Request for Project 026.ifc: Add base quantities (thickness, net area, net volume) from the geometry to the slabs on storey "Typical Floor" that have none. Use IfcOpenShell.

First a look at what the model holds.

```python
import ifcopenshell
import ifcopenshell.util.element
import ifcopenshell.util.unit

model = ifcopenshell.open("Project 026.ifc")
print(model.schema)
for unit_type in ("LENGTHUNIT", "AREAUNIT", "VOLUMEUNIT"):
    print(unit_type, ifcopenshell.util.unit.calculate_unit_scale(model, unit_type))
storey = next(s for s in model.by_type("IfcBuildingStorey") if s.Name == "Typical Floor")
slabs = [e for e in ifcopenshell.util.element.get_decomposition(storey) if e.is_a("IfcSlab")]
for e in sorted(slabs, key=lambda e: e.id()):
    print(e.id(), e.is_a(), e.Name, list(ifcopenshell.util.element.get_psets(e, qtos_only=True)), sep=" | ")
```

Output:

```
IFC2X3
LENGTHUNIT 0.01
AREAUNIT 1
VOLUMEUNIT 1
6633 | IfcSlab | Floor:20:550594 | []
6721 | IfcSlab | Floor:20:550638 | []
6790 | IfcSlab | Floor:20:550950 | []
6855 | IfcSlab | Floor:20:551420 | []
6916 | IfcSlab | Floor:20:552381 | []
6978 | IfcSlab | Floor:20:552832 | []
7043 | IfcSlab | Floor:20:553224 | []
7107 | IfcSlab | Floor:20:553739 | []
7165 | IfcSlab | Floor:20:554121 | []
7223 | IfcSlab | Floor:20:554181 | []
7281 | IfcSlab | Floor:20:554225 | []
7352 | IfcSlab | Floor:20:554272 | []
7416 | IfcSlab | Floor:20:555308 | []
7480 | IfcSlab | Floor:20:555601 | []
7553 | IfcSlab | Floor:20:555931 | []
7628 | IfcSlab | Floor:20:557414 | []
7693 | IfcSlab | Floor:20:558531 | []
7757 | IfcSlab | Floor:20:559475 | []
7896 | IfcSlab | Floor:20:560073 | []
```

```python
import ifcopenshell
import ifcopenshell.api.pset
import ifcopenshell.geom
import ifcopenshell.util.element
import ifcopenshell.util.shape
import ifcopenshell.util.unit

model = ifcopenshell.open("Project 026.ifc")
unit_scale = ifcopenshell.util.unit.calculate_unit_scale(model)
area_scale = ifcopenshell.util.unit.calculate_unit_scale(model, "AREAUNIT")
volume_scale = ifcopenshell.util.unit.calculate_unit_scale(model, "VOLUMEUNIT")
settings = ifcopenshell.geom.settings()

storey = next(s for s in model.by_type("IfcBuildingStorey") if s.Name == "Typical Floor")
slabs = [e for e in ifcopenshell.util.element.get_decomposition(storey) if e.is_a("IfcSlab")]

for e in sorted(slabs, key=lambda e: e.id()):
    if ifcopenshell.util.element.get_psets(e, qtos_only=True, should_inherit=False):
        continue
    # Geometry comes back in metres, in the element's own axes.
    shape = ifcopenshell.geom.create_shape(settings, e)
    values = {
        "Width": ifcopenshell.util.shape.get_z(shape.geometry) / unit_scale,
        "NetArea": ifcopenshell.util.shape.get_footprint_area(shape.geometry) / area_scale,
        "NetVolume": ifcopenshell.util.shape.get_volume(shape.geometry) / volume_scale,
    }
    qto = ifcopenshell.api.pset.add_qto(model, product=e, name="BaseQuantities")
    ifcopenshell.api.pset.edit_qto(model, qto=qto, properties=values)
    print(e.id(), {k: round(v, 3) for k, v in values.items()})

model.write("Project 026_edited.ifc")
```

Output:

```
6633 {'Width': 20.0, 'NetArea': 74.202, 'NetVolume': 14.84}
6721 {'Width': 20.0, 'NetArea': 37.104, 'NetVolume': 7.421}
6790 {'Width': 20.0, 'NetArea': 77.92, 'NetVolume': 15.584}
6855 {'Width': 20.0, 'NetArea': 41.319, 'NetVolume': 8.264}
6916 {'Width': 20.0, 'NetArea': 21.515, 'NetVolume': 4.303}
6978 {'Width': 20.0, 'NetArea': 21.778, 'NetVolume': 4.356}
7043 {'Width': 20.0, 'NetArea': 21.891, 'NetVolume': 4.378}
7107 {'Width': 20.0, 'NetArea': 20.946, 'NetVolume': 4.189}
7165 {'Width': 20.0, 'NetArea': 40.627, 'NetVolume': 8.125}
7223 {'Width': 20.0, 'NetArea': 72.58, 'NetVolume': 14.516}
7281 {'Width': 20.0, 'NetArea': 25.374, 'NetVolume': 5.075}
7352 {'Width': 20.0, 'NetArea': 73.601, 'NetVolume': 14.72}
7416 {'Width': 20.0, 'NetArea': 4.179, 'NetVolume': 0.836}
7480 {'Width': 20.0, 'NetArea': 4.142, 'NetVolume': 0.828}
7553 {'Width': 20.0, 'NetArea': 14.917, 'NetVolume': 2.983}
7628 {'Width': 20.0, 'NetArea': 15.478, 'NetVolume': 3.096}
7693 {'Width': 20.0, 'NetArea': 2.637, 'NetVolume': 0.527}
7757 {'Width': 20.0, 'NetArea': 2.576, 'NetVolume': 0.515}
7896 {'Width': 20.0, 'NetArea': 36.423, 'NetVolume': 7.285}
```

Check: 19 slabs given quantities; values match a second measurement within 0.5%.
